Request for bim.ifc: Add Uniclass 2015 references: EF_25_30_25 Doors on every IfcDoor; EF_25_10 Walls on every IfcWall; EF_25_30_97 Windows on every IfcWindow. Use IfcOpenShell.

First a look at what the model holds.

```python
import ifcopenshell

model = ifcopenshell.open("bim.ifc")
print(model.schema)
print("classifications:", [c.Name for c in model.by_type("IfcClassification")])
for ifc_class in ("IfcDoor", "IfcRoof", "IfcStair", "IfcWall", "IfcWindow"):
    print(ifc_class, len(model.by_type(ifc_class)))
```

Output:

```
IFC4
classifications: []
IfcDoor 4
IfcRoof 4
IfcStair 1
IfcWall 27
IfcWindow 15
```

```python
import ifcopenshell
import ifcopenshell.api.classification

model = ifcopenshell.open("bim.ifc")

system = ifcopenshell.api.classification.add_classification(model, classification="Uniclass 2015")

codes = {
    "IfcDoor": ("EF_25_30_25", "Doors"),
    "IfcWall": ("EF_25_10", "Walls"),
    "IfcWindow": ("EF_25_30_97", "Windows"),
}
for ifc_class, (code, name) in codes.items():
    products = model.by_type(ifc_class)
    ifcopenshell.api.classification.add_reference(
        model, products=products, classification=system, identification=code, name=name
    )
    print(code, len(products))

model.write("bim-out.ifc")
```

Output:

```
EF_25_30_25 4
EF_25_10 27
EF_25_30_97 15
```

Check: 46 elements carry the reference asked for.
